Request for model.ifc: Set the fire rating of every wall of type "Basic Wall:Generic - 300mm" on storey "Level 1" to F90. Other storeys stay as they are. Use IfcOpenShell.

First a look at what the model holds.

```python
import ifcopenshell
import ifcopenshell.util.element

model = ifcopenshell.open("model.ifc")
print(model.schema)
storey = next(s for s in model.by_type("IfcBuildingStorey") if s.Name == "Level 1")
walls = [e for e in ifcopenshell.util.element.get_decomposition(storey) if e.is_a("IfcWall")]
seen = {}
for e in walls:
    element_type = ifcopenshell.util.element.get_type(e)
    key = (element_type.Name if element_type != e and element_type else None, ifcopenshell.util.element.get_pset(e, "Pset_WallCommon", "FireRating"))
    seen[key] = seen.get(key, 0) + 1
for (name, value), count in sorted(seen.items(), key=str):
    print(count, "x", name, "|", value)
```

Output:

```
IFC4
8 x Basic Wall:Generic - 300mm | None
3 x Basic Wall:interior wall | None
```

```python
import ifcopenshell
import ifcopenshell.api.pset
import ifcopenshell.util.element

model = ifcopenshell.open("model.ifc")

storey = next(s for s in model.by_type("IfcBuildingStorey") if s.Name == "Level 1")
walls = [e for e in ifcopenshell.util.element.get_decomposition(storey) if e.is_a("IfcWall")]

count = 0
for e in walls:
    element_type = ifcopenshell.util.element.get_type(e)
    if element_type in (None, e) or element_type.Name != "Basic Wall:Generic - 300mm":
        continue
    # add_pset returns the element's existing set when there is one.
    pset = ifcopenshell.api.pset.add_pset(model, product=e, name="Pset_WallCommon")
    ifcopenshell.api.pset.edit_pset(model, pset=pset, properties={"FireRating": "F90"})
    count += 1

print(count, "walls updated")

model.write("model-out.ifc")
```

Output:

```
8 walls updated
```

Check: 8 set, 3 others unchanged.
